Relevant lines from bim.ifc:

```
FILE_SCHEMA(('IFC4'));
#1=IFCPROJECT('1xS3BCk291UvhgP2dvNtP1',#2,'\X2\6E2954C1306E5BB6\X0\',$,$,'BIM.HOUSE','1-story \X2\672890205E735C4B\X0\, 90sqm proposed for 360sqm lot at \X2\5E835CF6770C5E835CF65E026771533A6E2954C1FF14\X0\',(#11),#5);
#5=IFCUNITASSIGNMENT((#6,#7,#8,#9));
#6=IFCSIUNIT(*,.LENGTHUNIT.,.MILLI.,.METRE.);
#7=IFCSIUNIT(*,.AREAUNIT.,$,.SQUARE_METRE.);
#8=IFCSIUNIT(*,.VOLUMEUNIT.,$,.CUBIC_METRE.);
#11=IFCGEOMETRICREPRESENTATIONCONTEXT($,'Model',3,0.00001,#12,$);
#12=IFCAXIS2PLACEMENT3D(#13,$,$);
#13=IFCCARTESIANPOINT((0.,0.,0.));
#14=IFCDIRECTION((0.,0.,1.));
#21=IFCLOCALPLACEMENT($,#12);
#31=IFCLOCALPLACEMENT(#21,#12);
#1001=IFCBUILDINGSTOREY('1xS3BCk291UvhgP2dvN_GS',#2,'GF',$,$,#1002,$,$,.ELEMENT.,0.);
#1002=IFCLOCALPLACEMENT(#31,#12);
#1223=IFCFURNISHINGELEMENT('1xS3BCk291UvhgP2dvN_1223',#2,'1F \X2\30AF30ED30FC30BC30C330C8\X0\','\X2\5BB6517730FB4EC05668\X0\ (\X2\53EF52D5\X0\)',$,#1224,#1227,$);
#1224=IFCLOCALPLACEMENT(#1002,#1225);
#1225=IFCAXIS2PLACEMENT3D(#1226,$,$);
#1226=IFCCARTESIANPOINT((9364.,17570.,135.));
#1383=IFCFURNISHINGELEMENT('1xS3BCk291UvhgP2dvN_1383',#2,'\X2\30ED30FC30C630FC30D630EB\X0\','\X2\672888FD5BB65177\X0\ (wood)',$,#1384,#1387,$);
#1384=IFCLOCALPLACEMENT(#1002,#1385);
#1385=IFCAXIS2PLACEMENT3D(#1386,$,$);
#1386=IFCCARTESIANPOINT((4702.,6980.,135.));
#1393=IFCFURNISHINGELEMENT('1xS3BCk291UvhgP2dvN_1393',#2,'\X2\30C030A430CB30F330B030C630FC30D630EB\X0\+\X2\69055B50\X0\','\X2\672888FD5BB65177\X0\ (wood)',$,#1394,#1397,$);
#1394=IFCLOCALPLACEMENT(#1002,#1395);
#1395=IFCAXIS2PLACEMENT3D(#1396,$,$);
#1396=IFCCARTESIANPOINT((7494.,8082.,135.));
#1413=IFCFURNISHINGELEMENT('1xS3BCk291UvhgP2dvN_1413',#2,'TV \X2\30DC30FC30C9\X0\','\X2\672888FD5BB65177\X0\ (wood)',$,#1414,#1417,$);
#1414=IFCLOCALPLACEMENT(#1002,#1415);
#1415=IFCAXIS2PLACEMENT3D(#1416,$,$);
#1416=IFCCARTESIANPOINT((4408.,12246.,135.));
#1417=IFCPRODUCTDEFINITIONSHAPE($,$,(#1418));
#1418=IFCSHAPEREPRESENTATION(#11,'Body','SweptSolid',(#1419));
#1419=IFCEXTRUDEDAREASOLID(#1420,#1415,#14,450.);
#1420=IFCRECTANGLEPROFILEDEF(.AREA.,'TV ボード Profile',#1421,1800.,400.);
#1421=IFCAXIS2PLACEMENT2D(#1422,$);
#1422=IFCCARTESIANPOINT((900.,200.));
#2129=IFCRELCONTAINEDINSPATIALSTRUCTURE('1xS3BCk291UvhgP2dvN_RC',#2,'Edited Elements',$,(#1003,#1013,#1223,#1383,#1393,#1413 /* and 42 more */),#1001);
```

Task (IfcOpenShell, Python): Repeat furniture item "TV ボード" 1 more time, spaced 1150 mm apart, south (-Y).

```python
import numpy as np
import ifcopenshell
import ifcopenshell.api.geometry
import ifcopenshell.api.root
import ifcopenshell.util.element
import ifcopenshell.util.placement

model = ifcopenshell.open("bim.ifc")


def reuse_history(source, copy):
    """copy_class also copies each property set's owner history, people and application; keep the originals."""
    for rel in copy.IsDefinedBy:
        if rel.is_a("IfcRelDefinesByProperties") and (history := rel.RelatingPropertyDefinition.OwnerHistory):
            rel.RelatingPropertyDefinition.OwnerHistory = source.OwnerHistory
            ifcopenshell.util.element.remove_deep2(model, history)


source = model.by_guid("1xS3BCk291UvhgP2dvN_1413")
base = ifcopenshell.util.placement.get_local_placement(source.ObjectPlacement)
step = np.array([0.0, -1.0, 0.0]) * 1150.0

for i in range(1, 2):
    copy = ifcopenshell.api.root.copy_class(model, product=source)
    copy.Representation = ifcopenshell.util.element.copy_deep(
        model, source.Representation, exclude=["IfcGeometricRepresentationContext", "IfcRepresentationMap"]
    )
    reuse_history(source, copy)
    matrix = base.copy()
    matrix[:3, 3] += i * step
    print("added at", matrix[:3, 3].round(3) + 0.0)
    ifcopenshell.api.geometry.edit_object_placement(model, product=copy, matrix=matrix, is_si=False)

model.write("bim_v2.ifc")
```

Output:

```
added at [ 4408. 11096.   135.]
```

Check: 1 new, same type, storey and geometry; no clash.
